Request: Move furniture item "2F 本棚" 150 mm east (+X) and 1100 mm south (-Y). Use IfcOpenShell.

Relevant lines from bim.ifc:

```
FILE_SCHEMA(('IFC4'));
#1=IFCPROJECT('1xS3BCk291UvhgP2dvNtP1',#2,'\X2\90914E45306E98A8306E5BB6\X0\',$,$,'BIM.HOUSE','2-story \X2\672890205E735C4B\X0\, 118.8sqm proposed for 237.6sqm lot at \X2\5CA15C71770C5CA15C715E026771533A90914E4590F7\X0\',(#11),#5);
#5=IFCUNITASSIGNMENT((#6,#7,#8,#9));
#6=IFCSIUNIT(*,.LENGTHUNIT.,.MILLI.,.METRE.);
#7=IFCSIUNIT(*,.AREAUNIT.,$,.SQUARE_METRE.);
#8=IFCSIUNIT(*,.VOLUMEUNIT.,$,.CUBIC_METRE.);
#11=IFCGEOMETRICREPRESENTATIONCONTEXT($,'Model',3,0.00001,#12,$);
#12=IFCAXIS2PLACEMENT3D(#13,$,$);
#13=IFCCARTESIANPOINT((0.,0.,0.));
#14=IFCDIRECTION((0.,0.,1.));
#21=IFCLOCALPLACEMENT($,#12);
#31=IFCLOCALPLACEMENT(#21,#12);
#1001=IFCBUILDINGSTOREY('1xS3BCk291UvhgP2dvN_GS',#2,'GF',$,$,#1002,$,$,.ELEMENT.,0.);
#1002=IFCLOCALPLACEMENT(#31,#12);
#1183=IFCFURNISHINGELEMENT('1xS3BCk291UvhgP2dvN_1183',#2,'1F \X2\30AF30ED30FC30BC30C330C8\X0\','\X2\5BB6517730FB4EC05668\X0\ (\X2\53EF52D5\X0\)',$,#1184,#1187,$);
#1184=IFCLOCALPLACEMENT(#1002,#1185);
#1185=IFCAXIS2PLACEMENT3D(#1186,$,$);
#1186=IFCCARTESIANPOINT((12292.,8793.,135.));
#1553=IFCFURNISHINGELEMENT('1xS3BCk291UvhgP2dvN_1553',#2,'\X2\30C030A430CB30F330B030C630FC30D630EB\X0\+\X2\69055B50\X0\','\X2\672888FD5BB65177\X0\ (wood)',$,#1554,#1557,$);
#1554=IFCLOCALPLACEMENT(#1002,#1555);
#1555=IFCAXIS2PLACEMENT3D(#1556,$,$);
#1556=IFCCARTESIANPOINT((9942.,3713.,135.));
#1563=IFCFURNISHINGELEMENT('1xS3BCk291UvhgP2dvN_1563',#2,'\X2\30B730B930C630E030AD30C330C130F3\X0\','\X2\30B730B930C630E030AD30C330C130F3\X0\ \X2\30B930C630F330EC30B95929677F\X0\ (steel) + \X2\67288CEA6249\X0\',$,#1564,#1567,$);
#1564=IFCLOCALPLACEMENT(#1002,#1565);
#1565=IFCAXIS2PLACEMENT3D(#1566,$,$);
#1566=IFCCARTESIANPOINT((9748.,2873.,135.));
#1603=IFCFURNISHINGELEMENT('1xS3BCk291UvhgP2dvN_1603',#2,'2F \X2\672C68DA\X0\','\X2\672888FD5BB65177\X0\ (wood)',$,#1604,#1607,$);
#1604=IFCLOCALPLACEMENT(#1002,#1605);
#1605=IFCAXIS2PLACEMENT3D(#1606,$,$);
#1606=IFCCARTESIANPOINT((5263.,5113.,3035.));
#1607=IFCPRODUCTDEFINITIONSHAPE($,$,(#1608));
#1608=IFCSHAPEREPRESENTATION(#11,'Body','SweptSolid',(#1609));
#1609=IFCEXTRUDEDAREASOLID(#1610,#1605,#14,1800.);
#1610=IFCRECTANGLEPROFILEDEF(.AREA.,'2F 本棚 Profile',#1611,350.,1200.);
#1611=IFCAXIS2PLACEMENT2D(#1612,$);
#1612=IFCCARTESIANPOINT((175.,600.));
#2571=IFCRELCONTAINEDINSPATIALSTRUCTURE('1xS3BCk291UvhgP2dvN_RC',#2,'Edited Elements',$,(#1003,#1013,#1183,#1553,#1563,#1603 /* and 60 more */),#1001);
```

```python
import ifcopenshell
import ifcopenshell.api.geometry
import ifcopenshell.util.placement
import ifcopenshell.util.unit

model = ifcopenshell.open("bim.ifc")
unit_scale = ifcopenshell.util.unit.calculate_unit_scale(model)

item = model.by_guid("1xS3BCk291UvhgP2dvN_1603")
matrix = ifcopenshell.util.placement.get_local_placement(item.ObjectPlacement)
matrix[0, 3] += 0.15 / unit_scale
matrix[1, 3] -= 1.1 / unit_scale
ifcopenshell.api.geometry.edit_object_placement(model, product=item, matrix=matrix, is_si=False)

print(ifcopenshell.util.placement.get_local_placement(item.ObjectPlacement).round(3) + 0.0)

model.write("bim_edited.ifc")
```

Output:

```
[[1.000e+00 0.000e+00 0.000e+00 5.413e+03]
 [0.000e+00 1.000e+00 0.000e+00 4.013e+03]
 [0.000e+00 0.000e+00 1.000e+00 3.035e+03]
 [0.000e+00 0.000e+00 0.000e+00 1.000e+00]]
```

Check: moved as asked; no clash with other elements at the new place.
